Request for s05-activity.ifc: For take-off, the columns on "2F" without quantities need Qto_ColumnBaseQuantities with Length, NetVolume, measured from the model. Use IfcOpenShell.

First a look at what the model holds.

```python
import ifcopenshell
import ifcopenshell.util.element
import ifcopenshell.util.unit

model = ifcopenshell.open("s05-activity.ifc")
print(model.schema)
for unit_type in ("LENGTHUNIT", "AREAUNIT", "VOLUMEUNIT"):
    print(unit_type, ifcopenshell.util.unit.calculate_unit_scale(model, unit_type))
storey = next(s for s in model.by_type("IfcBuildingStorey") if s.Name == "2F")
columns = [e for e in ifcopenshell.util.element.get_decomposition(storey) if e.is_a("IfcColumn")]
for e in sorted(columns, key=lambda e: e.id()):
    print(e.id(), e.is_a(), e.Name, list(ifcopenshell.util.element.get_psets(e, qtos_only=True)), sep=" | ")
```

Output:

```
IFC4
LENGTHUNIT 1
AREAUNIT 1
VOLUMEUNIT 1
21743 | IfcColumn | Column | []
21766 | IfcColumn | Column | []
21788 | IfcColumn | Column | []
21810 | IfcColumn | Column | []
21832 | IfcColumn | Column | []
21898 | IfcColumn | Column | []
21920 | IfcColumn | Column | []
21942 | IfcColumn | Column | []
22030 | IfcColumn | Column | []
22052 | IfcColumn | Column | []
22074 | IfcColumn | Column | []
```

```python
import ifcopenshell
import ifcopenshell.api.pset
import ifcopenshell.geom
import ifcopenshell.util.element
import ifcopenshell.util.shape
import ifcopenshell.util.unit

model = ifcopenshell.open("s05-activity.ifc")
unit_scale = ifcopenshell.util.unit.calculate_unit_scale(model)
volume_scale = ifcopenshell.util.unit.calculate_unit_scale(model, "VOLUMEUNIT")
settings = ifcopenshell.geom.settings()

storey = next(s for s in model.by_type("IfcBuildingStorey") if s.Name == "2F")
columns = [e for e in ifcopenshell.util.element.get_decomposition(storey) if e.is_a("IfcColumn")]

for e in sorted(columns, key=lambda e: e.id()):
    if ifcopenshell.util.element.get_psets(e, qtos_only=True, should_inherit=False):
        continue
    # Geometry comes back in metres, in the element's own axes.
    shape = ifcopenshell.geom.create_shape(settings, e)
    values = {
        "Length": ifcopenshell.util.shape.get_z(shape.geometry) / unit_scale,
        "NetVolume": ifcopenshell.util.shape.get_volume(shape.geometry) / volume_scale,
    }
    qto = ifcopenshell.api.pset.add_qto(model, product=e, name="Qto_ColumnBaseQuantities")
    ifcopenshell.api.pset.edit_qto(model, qto=qto, properties=values)
    print(e.id(), {k: round(v, 3) for k, v in values.items()})

model.write("s05-activity_rev.ifc")
```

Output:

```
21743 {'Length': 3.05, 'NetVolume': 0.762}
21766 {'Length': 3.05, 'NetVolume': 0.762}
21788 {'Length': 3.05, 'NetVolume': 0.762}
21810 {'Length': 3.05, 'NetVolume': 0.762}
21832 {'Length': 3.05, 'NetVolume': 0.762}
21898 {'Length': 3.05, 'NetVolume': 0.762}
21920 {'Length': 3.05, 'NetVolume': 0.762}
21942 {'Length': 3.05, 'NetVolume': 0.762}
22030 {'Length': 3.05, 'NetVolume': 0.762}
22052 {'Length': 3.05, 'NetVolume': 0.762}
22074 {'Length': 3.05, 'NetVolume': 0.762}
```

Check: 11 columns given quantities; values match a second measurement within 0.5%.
